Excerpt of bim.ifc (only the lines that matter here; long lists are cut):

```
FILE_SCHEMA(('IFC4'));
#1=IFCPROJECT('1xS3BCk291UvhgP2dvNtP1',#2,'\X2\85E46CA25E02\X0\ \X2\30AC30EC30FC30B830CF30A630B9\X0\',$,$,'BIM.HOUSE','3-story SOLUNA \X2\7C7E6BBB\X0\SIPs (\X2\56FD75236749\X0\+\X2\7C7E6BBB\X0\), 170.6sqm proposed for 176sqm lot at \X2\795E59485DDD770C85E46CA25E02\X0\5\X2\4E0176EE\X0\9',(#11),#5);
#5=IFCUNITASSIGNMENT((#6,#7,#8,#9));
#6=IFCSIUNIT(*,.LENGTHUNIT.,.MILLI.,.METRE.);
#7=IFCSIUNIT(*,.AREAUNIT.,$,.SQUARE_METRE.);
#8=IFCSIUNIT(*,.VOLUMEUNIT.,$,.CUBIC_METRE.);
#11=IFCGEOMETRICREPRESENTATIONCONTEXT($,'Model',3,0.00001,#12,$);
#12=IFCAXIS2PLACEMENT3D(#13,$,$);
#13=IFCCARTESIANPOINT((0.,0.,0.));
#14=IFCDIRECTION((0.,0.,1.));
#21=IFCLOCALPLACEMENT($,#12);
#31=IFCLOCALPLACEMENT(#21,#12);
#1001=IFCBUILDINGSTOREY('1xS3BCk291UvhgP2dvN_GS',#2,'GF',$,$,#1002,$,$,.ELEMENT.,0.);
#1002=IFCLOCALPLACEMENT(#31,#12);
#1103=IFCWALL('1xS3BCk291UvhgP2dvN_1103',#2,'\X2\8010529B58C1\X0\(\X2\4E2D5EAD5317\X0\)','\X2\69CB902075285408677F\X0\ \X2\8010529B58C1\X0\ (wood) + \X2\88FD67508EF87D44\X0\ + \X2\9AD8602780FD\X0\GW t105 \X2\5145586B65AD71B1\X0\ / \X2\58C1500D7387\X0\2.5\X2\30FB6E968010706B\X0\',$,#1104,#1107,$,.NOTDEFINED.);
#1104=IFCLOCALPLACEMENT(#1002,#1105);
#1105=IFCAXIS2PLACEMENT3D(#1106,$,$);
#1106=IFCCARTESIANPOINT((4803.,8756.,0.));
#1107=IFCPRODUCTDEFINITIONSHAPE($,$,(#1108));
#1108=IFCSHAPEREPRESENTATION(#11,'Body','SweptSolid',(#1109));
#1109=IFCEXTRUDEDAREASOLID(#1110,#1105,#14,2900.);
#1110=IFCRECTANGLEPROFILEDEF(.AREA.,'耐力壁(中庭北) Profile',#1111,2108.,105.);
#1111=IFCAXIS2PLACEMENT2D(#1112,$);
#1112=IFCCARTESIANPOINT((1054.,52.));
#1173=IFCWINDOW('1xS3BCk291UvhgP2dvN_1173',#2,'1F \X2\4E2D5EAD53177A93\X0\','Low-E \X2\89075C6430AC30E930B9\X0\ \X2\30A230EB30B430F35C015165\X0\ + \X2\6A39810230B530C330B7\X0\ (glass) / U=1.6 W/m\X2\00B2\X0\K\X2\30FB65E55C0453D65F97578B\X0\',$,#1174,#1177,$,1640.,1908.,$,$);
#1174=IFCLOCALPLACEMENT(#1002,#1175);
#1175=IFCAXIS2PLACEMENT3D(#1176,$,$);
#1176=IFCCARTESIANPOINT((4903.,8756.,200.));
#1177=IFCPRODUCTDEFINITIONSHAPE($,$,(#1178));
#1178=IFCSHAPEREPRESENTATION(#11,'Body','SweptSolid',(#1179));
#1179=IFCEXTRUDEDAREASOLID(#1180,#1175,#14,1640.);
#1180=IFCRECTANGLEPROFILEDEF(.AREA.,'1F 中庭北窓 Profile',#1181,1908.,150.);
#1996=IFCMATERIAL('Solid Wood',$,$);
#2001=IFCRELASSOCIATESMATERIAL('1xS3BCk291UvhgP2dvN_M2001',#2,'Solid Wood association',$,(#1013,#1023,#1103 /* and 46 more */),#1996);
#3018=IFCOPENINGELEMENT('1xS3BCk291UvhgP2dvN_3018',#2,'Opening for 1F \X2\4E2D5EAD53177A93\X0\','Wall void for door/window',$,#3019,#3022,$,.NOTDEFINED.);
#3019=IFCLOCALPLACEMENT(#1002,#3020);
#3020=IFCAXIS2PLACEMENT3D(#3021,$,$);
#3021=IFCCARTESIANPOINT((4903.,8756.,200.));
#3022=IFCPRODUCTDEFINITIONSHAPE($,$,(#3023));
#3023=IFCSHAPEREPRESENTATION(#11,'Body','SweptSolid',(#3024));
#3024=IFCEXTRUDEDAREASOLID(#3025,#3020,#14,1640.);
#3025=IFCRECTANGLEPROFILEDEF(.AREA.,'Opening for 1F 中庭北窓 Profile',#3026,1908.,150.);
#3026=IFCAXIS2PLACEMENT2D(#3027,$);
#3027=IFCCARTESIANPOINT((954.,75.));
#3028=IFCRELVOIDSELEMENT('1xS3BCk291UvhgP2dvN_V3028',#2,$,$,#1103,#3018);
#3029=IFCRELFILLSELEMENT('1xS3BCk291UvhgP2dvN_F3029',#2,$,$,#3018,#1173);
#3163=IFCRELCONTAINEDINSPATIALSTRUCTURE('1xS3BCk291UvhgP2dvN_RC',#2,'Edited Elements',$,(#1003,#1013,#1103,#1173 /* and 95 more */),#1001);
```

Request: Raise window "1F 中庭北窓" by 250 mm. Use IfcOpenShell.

```python
import numpy as np
import ifcopenshell
import ifcopenshell.api.geometry
import ifcopenshell.util.placement
import ifcopenshell.util.unit

model = ifcopenshell.open("bim.ifc")
unit_scale = ifcopenshell.util.unit.calculate_unit_scale(model)

window = model.by_guid("1xS3BCk291UvhgP2dvN_1173")
opening = window.FillsVoids[0].RelatingOpeningElement
dz = 250.0

shift = np.array([0.0, 0.0, dz])
# The window is not placed relative to its opening, so move both.
for product in (opening, window):
    matrix = ifcopenshell.util.placement.get_local_placement(product.ObjectPlacement)
    matrix[:3, 3] += shift
    ifcopenshell.api.geometry.edit_object_placement(model, product=product, matrix=matrix, is_si=False)

print(f"moved by {dz * unit_scale:+.3f} m")

model.write("bim_rev.ifc")
```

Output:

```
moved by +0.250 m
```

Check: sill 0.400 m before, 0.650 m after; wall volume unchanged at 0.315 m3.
